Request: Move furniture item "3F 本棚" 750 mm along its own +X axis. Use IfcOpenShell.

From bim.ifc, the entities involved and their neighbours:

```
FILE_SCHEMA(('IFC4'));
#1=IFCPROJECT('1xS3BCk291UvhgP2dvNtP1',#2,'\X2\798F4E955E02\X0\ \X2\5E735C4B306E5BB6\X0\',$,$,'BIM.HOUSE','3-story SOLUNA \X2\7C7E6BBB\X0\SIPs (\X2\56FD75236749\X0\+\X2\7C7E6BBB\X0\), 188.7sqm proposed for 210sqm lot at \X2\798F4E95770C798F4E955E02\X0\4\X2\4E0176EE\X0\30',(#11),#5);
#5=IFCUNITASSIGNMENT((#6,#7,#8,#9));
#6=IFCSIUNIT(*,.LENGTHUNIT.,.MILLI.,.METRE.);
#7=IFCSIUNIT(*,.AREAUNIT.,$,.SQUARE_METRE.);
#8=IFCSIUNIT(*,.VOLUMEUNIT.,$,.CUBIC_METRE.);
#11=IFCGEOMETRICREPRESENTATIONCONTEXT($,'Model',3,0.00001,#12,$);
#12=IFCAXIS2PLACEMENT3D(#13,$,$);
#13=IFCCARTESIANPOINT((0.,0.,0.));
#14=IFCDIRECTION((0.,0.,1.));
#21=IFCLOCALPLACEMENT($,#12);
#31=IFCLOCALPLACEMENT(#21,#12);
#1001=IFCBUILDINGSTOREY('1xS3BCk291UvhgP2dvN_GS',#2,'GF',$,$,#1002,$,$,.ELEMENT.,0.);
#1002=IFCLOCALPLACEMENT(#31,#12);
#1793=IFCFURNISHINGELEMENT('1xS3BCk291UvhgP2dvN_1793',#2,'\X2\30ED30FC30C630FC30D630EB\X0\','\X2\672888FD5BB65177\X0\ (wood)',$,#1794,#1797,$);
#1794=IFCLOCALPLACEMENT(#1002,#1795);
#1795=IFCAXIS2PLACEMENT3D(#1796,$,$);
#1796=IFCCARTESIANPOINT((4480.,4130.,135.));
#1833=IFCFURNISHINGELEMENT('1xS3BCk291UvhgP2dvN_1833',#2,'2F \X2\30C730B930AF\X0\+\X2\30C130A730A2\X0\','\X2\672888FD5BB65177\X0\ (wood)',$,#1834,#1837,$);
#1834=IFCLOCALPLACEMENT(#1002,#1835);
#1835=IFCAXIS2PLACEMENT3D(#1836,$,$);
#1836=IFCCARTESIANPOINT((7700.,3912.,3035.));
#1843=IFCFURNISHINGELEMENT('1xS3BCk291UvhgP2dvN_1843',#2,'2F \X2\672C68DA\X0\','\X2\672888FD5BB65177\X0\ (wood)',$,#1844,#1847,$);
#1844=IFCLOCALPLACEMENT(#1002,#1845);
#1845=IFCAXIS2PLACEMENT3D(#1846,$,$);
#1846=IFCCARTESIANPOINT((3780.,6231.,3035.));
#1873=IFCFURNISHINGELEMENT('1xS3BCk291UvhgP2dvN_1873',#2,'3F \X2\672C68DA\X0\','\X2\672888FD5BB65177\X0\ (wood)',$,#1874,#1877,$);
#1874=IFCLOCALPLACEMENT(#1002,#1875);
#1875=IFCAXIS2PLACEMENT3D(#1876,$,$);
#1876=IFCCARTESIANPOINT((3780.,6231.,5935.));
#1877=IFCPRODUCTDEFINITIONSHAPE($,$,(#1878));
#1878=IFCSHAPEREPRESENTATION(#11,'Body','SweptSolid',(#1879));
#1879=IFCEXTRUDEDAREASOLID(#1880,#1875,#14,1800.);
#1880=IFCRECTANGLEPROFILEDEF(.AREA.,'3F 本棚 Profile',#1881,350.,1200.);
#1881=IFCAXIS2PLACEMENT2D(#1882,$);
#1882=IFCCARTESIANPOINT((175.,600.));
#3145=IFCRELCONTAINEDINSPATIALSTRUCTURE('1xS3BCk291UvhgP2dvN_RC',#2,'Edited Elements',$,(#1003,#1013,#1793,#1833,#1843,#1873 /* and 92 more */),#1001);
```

```python
import ifcopenshell
import ifcopenshell.api.geometry
import ifcopenshell.util.placement
import ifcopenshell.util.unit

model = ifcopenshell.open("bim.ifc")
unit_scale = ifcopenshell.util.unit.calculate_unit_scale(model)

item = model.by_guid("1xS3BCk291UvhgP2dvN_1873")
matrix = ifcopenshell.util.placement.get_local_placement(item.ObjectPlacement)
matrix[:3, 3] += matrix[:3, 0] * 0.75 / unit_scale
ifcopenshell.api.geometry.edit_object_placement(model, product=item, matrix=matrix, is_si=False)

print(ifcopenshell.util.placement.get_local_placement(item.ObjectPlacement).round(3) + 0.0)

model.write("bim_v2.ifc")
```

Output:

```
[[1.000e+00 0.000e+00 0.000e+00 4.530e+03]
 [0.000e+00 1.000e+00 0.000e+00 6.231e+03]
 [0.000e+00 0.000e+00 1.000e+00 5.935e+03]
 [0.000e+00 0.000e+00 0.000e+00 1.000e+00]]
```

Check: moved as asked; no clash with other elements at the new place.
